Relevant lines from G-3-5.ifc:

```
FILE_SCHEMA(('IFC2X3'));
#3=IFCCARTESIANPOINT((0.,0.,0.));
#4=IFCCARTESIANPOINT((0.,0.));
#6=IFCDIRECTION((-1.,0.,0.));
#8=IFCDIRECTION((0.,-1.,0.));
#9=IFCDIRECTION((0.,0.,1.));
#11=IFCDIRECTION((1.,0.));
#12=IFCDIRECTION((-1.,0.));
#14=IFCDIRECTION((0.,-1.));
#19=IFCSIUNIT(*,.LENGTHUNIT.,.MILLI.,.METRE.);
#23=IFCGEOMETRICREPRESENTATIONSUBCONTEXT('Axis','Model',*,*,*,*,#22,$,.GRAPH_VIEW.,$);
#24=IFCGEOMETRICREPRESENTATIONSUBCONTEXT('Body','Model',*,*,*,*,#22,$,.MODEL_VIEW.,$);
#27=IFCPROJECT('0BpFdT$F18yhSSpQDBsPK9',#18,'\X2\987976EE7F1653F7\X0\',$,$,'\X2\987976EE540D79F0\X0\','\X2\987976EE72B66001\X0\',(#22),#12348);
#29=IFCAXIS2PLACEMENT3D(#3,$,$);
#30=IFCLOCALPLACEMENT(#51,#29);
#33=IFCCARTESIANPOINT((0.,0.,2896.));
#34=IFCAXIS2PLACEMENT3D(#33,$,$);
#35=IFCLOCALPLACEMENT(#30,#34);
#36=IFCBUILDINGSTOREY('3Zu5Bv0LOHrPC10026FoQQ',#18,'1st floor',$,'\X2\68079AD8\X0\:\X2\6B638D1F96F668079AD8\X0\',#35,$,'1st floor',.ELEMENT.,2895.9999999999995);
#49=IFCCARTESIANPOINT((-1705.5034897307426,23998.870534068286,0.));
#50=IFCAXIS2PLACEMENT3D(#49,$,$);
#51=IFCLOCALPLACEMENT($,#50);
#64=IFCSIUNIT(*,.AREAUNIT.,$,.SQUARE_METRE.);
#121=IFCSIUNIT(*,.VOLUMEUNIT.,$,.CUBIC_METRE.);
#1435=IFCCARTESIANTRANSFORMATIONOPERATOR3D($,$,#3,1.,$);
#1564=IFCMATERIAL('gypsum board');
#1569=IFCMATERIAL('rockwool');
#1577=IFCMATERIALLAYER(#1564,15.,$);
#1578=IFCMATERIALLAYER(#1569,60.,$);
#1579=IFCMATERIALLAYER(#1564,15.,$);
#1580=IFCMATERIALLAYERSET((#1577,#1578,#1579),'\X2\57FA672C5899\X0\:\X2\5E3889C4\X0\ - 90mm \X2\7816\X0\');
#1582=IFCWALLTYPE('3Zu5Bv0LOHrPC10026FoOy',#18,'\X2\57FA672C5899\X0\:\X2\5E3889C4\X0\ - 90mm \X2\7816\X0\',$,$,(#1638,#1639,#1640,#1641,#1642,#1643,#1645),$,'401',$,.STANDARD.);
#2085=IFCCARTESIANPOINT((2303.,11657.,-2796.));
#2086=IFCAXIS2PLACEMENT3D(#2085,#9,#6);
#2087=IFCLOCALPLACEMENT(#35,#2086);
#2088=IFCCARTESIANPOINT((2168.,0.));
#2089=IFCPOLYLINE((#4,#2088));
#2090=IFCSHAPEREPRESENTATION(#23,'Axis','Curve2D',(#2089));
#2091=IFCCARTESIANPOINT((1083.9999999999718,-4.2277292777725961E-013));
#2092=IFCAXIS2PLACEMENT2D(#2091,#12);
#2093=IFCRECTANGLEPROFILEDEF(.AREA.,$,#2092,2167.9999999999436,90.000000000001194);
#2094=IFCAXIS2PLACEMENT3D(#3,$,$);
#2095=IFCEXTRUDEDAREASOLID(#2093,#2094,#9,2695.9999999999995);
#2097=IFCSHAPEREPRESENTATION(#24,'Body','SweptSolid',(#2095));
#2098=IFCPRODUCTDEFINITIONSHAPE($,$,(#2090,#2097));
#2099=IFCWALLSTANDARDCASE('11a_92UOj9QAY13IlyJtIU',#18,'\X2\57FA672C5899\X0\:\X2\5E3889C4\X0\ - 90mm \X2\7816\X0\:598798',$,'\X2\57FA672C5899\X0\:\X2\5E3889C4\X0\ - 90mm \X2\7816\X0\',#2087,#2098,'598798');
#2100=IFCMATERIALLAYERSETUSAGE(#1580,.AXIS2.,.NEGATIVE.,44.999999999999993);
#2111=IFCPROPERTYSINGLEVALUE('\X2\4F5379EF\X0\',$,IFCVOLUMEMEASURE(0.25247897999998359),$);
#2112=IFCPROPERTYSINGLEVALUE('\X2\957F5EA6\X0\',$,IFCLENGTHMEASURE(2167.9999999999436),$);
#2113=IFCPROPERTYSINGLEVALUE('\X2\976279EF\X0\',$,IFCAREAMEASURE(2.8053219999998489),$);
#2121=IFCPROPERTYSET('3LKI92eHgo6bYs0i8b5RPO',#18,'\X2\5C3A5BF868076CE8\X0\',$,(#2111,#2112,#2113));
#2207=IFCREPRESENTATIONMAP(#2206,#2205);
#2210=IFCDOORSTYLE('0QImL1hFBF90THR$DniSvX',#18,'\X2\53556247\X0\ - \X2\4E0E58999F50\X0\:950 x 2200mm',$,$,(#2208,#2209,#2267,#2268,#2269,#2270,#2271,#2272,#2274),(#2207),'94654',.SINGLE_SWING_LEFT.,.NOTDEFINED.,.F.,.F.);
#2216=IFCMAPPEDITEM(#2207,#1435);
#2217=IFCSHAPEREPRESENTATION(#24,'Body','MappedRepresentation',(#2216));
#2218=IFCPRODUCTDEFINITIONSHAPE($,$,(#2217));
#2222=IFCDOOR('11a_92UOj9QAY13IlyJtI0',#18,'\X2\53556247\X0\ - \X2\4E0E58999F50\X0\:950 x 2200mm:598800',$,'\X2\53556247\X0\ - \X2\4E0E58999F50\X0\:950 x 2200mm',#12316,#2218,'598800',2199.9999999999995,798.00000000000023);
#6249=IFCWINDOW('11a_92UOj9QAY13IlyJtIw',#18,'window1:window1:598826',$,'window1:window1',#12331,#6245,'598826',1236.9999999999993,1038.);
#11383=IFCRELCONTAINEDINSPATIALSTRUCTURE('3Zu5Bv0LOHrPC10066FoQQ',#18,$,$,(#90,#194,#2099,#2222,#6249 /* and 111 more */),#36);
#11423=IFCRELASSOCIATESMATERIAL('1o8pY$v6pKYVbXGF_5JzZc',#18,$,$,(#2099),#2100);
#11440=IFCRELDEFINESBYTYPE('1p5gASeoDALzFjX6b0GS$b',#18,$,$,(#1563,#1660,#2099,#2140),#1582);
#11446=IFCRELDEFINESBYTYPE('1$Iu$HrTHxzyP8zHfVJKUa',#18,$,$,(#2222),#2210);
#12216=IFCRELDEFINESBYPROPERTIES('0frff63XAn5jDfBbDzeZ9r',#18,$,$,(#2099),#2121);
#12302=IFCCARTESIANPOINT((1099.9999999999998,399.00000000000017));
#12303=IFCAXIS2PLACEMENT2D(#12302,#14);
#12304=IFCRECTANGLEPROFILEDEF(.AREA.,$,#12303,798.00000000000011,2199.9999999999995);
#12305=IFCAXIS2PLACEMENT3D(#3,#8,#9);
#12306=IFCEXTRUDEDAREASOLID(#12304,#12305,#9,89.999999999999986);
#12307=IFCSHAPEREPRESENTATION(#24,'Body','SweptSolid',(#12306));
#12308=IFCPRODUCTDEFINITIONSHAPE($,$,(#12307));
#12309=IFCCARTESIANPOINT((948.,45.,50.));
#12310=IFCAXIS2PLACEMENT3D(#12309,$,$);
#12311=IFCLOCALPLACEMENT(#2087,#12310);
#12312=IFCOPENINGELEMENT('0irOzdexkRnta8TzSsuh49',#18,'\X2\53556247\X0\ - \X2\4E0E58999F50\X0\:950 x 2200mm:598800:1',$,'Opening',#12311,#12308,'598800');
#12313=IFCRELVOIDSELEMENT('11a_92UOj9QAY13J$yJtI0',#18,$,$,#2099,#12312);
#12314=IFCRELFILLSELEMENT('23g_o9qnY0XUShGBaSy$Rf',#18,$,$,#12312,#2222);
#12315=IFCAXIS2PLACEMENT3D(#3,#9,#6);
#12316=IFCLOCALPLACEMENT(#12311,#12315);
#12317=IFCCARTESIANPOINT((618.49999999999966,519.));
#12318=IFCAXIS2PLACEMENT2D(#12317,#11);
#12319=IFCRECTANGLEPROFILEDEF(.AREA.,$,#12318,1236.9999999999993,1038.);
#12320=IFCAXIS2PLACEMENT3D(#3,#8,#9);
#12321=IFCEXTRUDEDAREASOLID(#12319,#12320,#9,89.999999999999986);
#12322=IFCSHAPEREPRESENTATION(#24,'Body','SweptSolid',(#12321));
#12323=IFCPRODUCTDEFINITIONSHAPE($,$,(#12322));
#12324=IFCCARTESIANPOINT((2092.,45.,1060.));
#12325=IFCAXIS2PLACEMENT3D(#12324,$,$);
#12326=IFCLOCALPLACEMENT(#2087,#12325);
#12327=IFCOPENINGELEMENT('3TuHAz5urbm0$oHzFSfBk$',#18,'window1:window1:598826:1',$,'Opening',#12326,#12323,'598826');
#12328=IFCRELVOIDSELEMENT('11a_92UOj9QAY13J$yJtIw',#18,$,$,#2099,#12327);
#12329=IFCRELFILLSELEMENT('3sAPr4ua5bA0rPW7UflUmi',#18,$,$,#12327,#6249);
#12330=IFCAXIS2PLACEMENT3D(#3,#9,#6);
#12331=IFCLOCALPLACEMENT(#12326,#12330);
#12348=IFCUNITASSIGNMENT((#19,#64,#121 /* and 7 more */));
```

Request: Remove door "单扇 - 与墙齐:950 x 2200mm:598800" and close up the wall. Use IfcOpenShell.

```python
import ifcopenshell
import ifcopenshell.api.feature
import ifcopenshell.api.pset
import ifcopenshell.api.root
import ifcopenshell.geom
import ifcopenshell.util.element
import ifcopenshell.util.shape
import ifcopenshell.util.unit

model = ifcopenshell.open("G-3-5.ifc")
area_scale = ifcopenshell.util.unit.calculate_unit_scale(model, "AREAUNIT")
volume_scale = ifcopenshell.util.unit.calculate_unit_scale(model, "VOLUMEUNIT")
settings = ifcopenshell.geom.settings()


def volume(element):
    """Net volume in cubic metres, openings subtracted."""
    shape = ifcopenshell.geom.create_shape(settings, element)
    return ifcopenshell.util.shape.get_volume(shape.geometry)


door = model.by_id(2222)
opening = door.FillsVoids[0].RelatingOpeningElement
wall = opening.VoidsElements[0].RelatingBuildingElement
before = volume(wall)

ifcopenshell.api.root.remove_product(model, product=door)
ifcopenshell.api.feature.remove_feature(model, feature=opening)

after = volume(wall)
thickness = 0.09  # wall thickness in metres

# Update the wall's stored quantities.
pset = model.by_id(ifcopenshell.util.element.get_pset(wall, "尺寸标注", should_inherit=False)["id"])
ifcopenshell.api.pset.edit_pset(model, pset=pset, properties={
    "体积": model.create_entity("IfcVolumeMeasure", after / volume_scale),
    "面积": model.create_entity("IfcAreaMeasure", after / thickness / area_scale),
})

print(f"wall volume {before:.3f} -> {after:.3f} m3")

model.write("G-3-5_v2.ifc")
```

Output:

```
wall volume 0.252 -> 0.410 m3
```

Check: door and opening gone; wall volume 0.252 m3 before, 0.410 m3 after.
